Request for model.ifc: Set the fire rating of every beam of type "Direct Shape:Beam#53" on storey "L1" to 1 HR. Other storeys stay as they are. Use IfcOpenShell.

First a look at what the model holds.

```python
import ifcopenshell
import ifcopenshell.util.element

model = ifcopenshell.open("model.ifc")
print(model.schema)
storey = next(s for s in model.by_type("IfcBuildingStorey") if s.Name == "L1")
beams = [e for e in ifcopenshell.util.element.get_decomposition(storey) if e.is_a("IfcBeam")]
seen = {}
for e in beams:
    element_type = ifcopenshell.util.element.get_type(e)
    key = (element_type.Name if element_type != e and element_type else None, ifcopenshell.util.element.get_pset(e, "Pset_BeamCommon", "FireRating"))
    seen[key] = seen.get(key, 0) + 1
for (name, value), count in sorted(seen.items(), key=str):
    print(count, "x", name, "|", value)
```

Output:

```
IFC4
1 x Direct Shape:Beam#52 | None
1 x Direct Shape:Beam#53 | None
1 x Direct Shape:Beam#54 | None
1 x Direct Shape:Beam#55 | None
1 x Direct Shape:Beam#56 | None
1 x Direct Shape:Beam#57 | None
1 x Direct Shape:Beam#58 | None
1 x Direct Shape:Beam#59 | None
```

```python
import ifcopenshell
import ifcopenshell.api.pset
import ifcopenshell.util.element

model = ifcopenshell.open("model.ifc")

storey = next(s for s in model.by_type("IfcBuildingStorey") if s.Name == "L1")
beams = [e for e in ifcopenshell.util.element.get_decomposition(storey) if e.is_a("IfcBeam")]

count = 0
for e in beams:
    element_type = ifcopenshell.util.element.get_type(e)
    if element_type in (None, e) or element_type.Name != "Direct Shape:Beam#53":
        continue
    # add_pset returns the element's existing set when there is one.
    pset = ifcopenshell.api.pset.add_pset(model, product=e, name="Pset_BeamCommon")
    ifcopenshell.api.pset.edit_pset(model, pset=pset, properties={"FireRating": "1 HR"})
    count += 1

print(count, "beams updated")

model.write("model_v2.ifc")
```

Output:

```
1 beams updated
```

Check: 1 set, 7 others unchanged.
